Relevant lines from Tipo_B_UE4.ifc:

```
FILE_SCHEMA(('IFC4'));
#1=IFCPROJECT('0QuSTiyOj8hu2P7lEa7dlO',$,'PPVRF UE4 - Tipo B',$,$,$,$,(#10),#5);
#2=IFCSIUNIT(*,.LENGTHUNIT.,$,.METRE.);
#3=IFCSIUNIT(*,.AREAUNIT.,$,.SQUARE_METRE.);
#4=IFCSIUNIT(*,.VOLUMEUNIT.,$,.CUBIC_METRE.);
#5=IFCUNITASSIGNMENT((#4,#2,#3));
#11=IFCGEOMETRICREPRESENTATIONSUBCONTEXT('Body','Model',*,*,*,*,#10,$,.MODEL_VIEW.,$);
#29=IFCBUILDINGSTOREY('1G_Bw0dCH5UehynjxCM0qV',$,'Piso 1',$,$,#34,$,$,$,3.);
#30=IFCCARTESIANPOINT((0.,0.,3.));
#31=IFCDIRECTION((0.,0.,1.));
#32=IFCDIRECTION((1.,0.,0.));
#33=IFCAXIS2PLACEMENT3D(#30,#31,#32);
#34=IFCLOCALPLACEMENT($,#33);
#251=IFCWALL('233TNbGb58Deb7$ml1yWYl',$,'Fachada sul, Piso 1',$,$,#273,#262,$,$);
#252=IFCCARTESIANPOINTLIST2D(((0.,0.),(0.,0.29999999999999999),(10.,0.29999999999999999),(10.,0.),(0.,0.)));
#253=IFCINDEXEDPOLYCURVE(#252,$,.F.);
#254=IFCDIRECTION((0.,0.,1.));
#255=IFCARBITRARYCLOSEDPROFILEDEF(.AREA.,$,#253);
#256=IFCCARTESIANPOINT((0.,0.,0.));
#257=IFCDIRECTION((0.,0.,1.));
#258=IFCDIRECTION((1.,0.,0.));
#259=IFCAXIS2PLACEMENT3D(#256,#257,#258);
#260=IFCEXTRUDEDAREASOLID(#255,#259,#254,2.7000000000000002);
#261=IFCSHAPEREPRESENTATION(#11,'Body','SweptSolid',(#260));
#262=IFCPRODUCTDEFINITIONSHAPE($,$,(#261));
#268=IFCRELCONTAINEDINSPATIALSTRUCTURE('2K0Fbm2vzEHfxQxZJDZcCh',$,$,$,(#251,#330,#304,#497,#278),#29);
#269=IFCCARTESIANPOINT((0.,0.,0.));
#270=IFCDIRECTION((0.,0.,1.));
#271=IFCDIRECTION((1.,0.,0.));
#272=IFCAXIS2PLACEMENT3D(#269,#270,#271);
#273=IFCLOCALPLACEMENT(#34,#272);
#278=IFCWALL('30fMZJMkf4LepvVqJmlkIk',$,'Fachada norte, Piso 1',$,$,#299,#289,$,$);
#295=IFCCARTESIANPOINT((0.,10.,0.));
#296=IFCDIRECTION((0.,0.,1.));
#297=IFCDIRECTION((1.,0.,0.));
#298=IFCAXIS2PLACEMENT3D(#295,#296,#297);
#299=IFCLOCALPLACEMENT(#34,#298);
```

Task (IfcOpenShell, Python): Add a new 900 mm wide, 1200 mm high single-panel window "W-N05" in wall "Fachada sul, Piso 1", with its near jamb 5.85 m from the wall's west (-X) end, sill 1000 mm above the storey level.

```python
import numpy as np
import ifcopenshell
import ifcopenshell.api.feature
import ifcopenshell.api.geometry
import ifcopenshell.api.root
import ifcopenshell.api.spatial
import ifcopenshell.geom
import ifcopenshell.util.element
import ifcopenshell.util.placement
import ifcopenshell.util.representation
import ifcopenshell.util.shape
import ifcopenshell.util.unit

model = ifcopenshell.open("Tipo_B_UE4.ifc")
unit_scale = ifcopenshell.util.unit.calculate_unit_scale(model)
settings = ifcopenshell.geom.settings()


def volume(element):
    """Net volume in cubic metres, openings subtracted."""
    shape = ifcopenshell.geom.create_shape(settings, element)
    return ifcopenshell.util.shape.get_volume(shape.geometry)


wall = model.by_id(251)
storey = ifcopenshell.util.element.get_container(wall, ifc_class="IfcBuildingStorey")
context = ifcopenshell.util.representation.get_context(model, "Model", "Body", "MODEL_VIEW")
before = volume(wall)

width, height, from_end, sill = 0.9, 1.2, 5.85, 1  # metres

# The wall runs along its own X axis, and the end named is its -X end.
wall_shape = ifcopenshell.geom.create_shape(settings, wall)
x, y, z = ifcopenshell.util.shape.get_vertices(wall_shape.geometry).T
start = x.min() + from_end
face, thickness = float(y.min()), float(y.max() - y.min())
wall_matrix = ifcopenshell.util.placement.get_local_placement(wall.ObjectPlacement)
level = ifcopenshell.util.placement.get_local_placement(storey.ObjectPlacement)[2, 3]


def in_wall(x, y):
    """Placement at x, y metres in the wall's axes, at sill height."""
    matrix = wall_matrix.copy()
    matrix[:, 3] = wall_matrix @ np.array([x / unit_scale, y / unit_scale, 0.0, 1.0])
    matrix[2, 3] = level + sill / unit_scale
    return matrix


# Opening: a box that overshoots both wall faces by 50 mm.
opening = ifcopenshell.api.root.create_entity(model, ifc_class="IfcOpeningElement", predefined_type="OPENING")
box = ifcopenshell.api.geometry.add_wall_representation(
    model, context=context, length=width, height=height, thickness=thickness + 0.1
)
ifcopenshell.api.geometry.assign_representation(model, product=opening, representation=box)
ifcopenshell.api.geometry.edit_object_placement(model, product=opening, matrix=in_wall(start, face - 0.05), is_si=False)
ifcopenshell.api.feature.add_feature(model, feature=opening, element=wall)

window = ifcopenshell.api.root.create_entity(model, ifc_class="IfcWindow", name="W-N05", predefined_type="WINDOW")
window.OverallWidth, window.OverallHeight = width / unit_scale, height / unit_scale
window.PartitioningType = "SINGLE_PANEL"
body = ifcopenshell.api.geometry.add_window_representation(
    model,
    context=context,
    overall_width=window.OverallWidth,
    overall_height=window.OverallHeight,
    partition_type="SINGLE_PANEL",
)
ifcopenshell.api.geometry.assign_representation(model, product=window, representation=body)
ifcopenshell.api.spatial.assign_container(model, products=[window], relating_structure=storey)
ifcopenshell.api.feature.add_filling(model, opening=opening, element=window)

# Centre the window in the wall's thickness.
ifcopenshell.api.geometry.edit_object_placement(model, product=window, matrix=in_wall(start, face), is_si=False)
window_shape = ifcopenshell.geom.create_shape(settings, window)
depth = ifcopenshell.util.shape.get_vertices(window_shape.geometry)[:, 1]
offset = face + thickness / 2 - (depth.min() + depth.max()) / 2
ifcopenshell.api.geometry.edit_object_placement(model, product=window, matrix=in_wall(start, offset), is_si=False)

after = volume(wall)

print(f"wall volume {before:.3f} -> {after:.3f} m3")

model.write("Tipo_B_UE4-out.ifc")
```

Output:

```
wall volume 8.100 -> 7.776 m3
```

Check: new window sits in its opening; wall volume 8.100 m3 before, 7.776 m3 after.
